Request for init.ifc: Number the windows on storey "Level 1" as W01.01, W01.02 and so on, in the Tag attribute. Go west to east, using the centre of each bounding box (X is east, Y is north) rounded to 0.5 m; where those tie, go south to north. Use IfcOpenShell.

First a look at what the model holds.

```python
import ifcopenshell
import ifcopenshell.util.element
import ifcopenshell.util.placement

model = ifcopenshell.open("init.ifc")
print(model.schema)
storey = next(s for s in model.by_type("IfcBuildingStorey") if s.Name == "Level 1")
windows = [e for e in ifcopenshell.util.element.get_decomposition(storey) if e.is_a("IfcWindow")]
for e in sorted(windows, key=lambda e: e.id()):
    origin = ifcopenshell.util.placement.get_local_placement(e.ObjectPlacement)[:3, 3]
    print(e.id(), e.Tag, e.Name, origin.round(2) + 0.0, sep=" | ")
```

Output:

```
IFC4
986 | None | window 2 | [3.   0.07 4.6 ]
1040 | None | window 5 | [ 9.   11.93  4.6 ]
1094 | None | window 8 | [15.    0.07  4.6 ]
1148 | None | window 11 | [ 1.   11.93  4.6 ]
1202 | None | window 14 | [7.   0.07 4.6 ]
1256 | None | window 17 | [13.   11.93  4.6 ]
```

```python
import ifcopenshell
import ifcopenshell.geom
import ifcopenshell.util.element
import ifcopenshell.util.shape

model = ifcopenshell.open("init.ifc")
settings = ifcopenshell.geom.settings()
settings.set("use-world-coords", True)


def centre(element):
    shape = ifcopenshell.geom.create_shape(settings, element)
    return ifcopenshell.util.shape.get_bbox_centroid(shape.geometry)


storey = next(s for s in model.by_type("IfcBuildingStorey") if s.Name == "Level 1")
windows = [e for e in ifcopenshell.util.element.get_decomposition(storey) if e.is_a("IfcWindow")]

# Insertion points can sit at a corner or the storey origin, so sort by the geometry (in metres).
centres = {e: centre(e) for e in windows}
windows.sort(key=lambda e: (round(centres[e][0] / 0.5), centres[e][1]))

for i, e in enumerate(windows, start=1):
    number = f"W01.{i:02d}"
    e.Tag = number
    print(e.id(), number)

model.write("init_edited.ifc")
```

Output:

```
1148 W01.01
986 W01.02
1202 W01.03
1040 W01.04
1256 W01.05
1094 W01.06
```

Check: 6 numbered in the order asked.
